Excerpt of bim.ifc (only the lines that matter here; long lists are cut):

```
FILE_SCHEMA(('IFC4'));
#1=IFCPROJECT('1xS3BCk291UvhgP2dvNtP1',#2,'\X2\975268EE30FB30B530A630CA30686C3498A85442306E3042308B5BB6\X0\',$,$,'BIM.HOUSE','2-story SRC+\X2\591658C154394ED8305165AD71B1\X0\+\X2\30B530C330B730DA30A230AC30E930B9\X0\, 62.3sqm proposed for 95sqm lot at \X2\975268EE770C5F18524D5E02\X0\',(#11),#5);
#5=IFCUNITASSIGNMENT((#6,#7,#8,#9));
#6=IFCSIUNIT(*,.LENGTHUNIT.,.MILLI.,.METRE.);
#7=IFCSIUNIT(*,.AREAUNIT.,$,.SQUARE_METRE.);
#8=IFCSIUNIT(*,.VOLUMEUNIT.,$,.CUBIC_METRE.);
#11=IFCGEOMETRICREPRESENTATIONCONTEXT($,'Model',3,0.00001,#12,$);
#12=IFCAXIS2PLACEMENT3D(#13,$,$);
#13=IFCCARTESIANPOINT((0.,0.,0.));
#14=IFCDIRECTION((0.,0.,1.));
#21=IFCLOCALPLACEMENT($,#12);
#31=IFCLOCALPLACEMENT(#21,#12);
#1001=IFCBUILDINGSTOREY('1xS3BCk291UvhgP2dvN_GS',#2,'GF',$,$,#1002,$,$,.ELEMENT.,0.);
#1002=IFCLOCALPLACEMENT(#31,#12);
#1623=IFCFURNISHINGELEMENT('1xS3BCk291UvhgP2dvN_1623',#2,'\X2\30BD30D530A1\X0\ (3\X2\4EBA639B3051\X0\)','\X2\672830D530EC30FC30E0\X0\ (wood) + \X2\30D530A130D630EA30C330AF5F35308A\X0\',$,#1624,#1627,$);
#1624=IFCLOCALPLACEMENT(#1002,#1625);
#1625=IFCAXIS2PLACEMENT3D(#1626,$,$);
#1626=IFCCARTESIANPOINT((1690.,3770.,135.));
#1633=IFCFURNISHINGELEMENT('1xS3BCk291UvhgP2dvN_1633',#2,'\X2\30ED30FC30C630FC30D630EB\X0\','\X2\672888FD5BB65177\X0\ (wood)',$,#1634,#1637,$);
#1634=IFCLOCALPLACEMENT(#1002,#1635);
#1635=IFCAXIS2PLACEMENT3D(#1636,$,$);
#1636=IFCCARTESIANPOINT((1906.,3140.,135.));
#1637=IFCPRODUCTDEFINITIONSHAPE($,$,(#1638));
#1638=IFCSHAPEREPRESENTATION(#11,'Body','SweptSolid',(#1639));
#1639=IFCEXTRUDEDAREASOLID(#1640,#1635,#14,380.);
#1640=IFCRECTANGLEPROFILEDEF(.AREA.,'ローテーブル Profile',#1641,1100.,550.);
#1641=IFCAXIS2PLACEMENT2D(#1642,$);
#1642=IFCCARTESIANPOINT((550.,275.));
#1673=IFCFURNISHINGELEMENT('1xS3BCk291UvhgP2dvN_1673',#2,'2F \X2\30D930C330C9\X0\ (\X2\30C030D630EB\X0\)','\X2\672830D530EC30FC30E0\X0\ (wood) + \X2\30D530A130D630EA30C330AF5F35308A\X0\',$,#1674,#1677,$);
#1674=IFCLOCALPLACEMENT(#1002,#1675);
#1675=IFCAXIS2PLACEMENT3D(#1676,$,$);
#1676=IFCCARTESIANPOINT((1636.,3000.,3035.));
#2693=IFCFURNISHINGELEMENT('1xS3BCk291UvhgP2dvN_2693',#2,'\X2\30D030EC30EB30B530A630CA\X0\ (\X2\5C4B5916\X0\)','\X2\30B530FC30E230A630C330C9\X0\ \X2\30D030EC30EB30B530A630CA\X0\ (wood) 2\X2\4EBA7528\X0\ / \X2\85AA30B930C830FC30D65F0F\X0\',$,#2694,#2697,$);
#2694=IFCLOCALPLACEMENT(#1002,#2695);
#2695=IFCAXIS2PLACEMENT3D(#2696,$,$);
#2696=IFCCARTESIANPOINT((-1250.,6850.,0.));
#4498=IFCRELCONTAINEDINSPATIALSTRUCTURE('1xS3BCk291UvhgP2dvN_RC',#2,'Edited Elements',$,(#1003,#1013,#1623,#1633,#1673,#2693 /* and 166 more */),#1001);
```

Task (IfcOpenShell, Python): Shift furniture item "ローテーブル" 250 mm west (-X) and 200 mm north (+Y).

```python
import ifcopenshell
import ifcopenshell.api.geometry
import ifcopenshell.util.placement
import ifcopenshell.util.unit

model = ifcopenshell.open("bim.ifc")
unit_scale = ifcopenshell.util.unit.calculate_unit_scale(model)

item = model.by_guid("1xS3BCk291UvhgP2dvN_1633")
matrix = ifcopenshell.util.placement.get_local_placement(item.ObjectPlacement)
matrix[0, 3] -= 0.25 / unit_scale
matrix[1, 3] += 0.2 / unit_scale
ifcopenshell.api.geometry.edit_object_placement(model, product=item, matrix=matrix, is_si=False)

print(ifcopenshell.util.placement.get_local_placement(item.ObjectPlacement).round(3) + 0.0)

model.write("bim_edited.ifc")
```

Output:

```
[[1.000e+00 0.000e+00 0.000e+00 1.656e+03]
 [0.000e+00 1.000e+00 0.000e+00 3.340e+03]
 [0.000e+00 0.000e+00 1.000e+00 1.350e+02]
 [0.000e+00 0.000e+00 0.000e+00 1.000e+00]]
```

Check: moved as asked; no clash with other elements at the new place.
